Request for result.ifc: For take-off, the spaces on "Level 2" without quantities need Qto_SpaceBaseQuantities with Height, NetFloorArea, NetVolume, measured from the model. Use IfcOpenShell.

First a look at what the model holds.

```python
import ifcopenshell
import ifcopenshell.util.element
import ifcopenshell.util.unit

model = ifcopenshell.open("result.ifc")
print(model.schema)
for unit_type in ("LENGTHUNIT", "AREAUNIT", "VOLUMEUNIT"):
    print(unit_type, ifcopenshell.util.unit.calculate_unit_scale(model, unit_type))
storey = next(s for s in model.by_type("IfcBuildingStorey") if s.Name == "Level 2")
spaces = [e for e in ifcopenshell.util.element.get_decomposition(storey) if e.is_a("IfcSpace")]
for e in sorted(spaces, key=lambda e: e.id()):
    print(e.id(), e.is_a(), e.Name, list(ifcopenshell.util.element.get_psets(e, qtos_only=True)), sep=" | ")
```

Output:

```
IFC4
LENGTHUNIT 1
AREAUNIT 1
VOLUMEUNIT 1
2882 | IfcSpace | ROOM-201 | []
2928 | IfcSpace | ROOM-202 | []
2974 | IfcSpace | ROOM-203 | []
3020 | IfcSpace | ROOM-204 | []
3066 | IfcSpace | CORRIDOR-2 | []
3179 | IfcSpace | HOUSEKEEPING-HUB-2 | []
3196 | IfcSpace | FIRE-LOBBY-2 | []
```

```python
import ifcopenshell
import ifcopenshell.api.pset
import ifcopenshell.geom
import ifcopenshell.util.element
import ifcopenshell.util.shape
import ifcopenshell.util.unit

model = ifcopenshell.open("result.ifc")
unit_scale = ifcopenshell.util.unit.calculate_unit_scale(model)
area_scale = ifcopenshell.util.unit.calculate_unit_scale(model, "AREAUNIT")
volume_scale = ifcopenshell.util.unit.calculate_unit_scale(model, "VOLUMEUNIT")
settings = ifcopenshell.geom.settings()

storey = next(s for s in model.by_type("IfcBuildingStorey") if s.Name == "Level 2")
spaces = [e for e in ifcopenshell.util.element.get_decomposition(storey) if e.is_a("IfcSpace")]

for e in sorted(spaces, key=lambda e: e.id()):
    if ifcopenshell.util.element.get_psets(e, qtos_only=True, should_inherit=False):
        continue
    # Geometry comes back in metres, in the element's own axes.
    shape = ifcopenshell.geom.create_shape(settings, e)
    values = {
        "Height": ifcopenshell.util.shape.get_z(shape.geometry) / unit_scale,
        "NetFloorArea": ifcopenshell.util.shape.get_footprint_area(shape.geometry) / area_scale,
        "NetVolume": ifcopenshell.util.shape.get_volume(shape.geometry) / volume_scale,
    }
    qto = ifcopenshell.api.pset.add_qto(model, product=e, name="Qto_SpaceBaseQuantities")
    ifcopenshell.api.pset.edit_qto(model, qto=qto, properties=values)
    print(e.id(), {k: round(v, 3) for k, v in values.items()})

model.write("result_edited.ifc")
```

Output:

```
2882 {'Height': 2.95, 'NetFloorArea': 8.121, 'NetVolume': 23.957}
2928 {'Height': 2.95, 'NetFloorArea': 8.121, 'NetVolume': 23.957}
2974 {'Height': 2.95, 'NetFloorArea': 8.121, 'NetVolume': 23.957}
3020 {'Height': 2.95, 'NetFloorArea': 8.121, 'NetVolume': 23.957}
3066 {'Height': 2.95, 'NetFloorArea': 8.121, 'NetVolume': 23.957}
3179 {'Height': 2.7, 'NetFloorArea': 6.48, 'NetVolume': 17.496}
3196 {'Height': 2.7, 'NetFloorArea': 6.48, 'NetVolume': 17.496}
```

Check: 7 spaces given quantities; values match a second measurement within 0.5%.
